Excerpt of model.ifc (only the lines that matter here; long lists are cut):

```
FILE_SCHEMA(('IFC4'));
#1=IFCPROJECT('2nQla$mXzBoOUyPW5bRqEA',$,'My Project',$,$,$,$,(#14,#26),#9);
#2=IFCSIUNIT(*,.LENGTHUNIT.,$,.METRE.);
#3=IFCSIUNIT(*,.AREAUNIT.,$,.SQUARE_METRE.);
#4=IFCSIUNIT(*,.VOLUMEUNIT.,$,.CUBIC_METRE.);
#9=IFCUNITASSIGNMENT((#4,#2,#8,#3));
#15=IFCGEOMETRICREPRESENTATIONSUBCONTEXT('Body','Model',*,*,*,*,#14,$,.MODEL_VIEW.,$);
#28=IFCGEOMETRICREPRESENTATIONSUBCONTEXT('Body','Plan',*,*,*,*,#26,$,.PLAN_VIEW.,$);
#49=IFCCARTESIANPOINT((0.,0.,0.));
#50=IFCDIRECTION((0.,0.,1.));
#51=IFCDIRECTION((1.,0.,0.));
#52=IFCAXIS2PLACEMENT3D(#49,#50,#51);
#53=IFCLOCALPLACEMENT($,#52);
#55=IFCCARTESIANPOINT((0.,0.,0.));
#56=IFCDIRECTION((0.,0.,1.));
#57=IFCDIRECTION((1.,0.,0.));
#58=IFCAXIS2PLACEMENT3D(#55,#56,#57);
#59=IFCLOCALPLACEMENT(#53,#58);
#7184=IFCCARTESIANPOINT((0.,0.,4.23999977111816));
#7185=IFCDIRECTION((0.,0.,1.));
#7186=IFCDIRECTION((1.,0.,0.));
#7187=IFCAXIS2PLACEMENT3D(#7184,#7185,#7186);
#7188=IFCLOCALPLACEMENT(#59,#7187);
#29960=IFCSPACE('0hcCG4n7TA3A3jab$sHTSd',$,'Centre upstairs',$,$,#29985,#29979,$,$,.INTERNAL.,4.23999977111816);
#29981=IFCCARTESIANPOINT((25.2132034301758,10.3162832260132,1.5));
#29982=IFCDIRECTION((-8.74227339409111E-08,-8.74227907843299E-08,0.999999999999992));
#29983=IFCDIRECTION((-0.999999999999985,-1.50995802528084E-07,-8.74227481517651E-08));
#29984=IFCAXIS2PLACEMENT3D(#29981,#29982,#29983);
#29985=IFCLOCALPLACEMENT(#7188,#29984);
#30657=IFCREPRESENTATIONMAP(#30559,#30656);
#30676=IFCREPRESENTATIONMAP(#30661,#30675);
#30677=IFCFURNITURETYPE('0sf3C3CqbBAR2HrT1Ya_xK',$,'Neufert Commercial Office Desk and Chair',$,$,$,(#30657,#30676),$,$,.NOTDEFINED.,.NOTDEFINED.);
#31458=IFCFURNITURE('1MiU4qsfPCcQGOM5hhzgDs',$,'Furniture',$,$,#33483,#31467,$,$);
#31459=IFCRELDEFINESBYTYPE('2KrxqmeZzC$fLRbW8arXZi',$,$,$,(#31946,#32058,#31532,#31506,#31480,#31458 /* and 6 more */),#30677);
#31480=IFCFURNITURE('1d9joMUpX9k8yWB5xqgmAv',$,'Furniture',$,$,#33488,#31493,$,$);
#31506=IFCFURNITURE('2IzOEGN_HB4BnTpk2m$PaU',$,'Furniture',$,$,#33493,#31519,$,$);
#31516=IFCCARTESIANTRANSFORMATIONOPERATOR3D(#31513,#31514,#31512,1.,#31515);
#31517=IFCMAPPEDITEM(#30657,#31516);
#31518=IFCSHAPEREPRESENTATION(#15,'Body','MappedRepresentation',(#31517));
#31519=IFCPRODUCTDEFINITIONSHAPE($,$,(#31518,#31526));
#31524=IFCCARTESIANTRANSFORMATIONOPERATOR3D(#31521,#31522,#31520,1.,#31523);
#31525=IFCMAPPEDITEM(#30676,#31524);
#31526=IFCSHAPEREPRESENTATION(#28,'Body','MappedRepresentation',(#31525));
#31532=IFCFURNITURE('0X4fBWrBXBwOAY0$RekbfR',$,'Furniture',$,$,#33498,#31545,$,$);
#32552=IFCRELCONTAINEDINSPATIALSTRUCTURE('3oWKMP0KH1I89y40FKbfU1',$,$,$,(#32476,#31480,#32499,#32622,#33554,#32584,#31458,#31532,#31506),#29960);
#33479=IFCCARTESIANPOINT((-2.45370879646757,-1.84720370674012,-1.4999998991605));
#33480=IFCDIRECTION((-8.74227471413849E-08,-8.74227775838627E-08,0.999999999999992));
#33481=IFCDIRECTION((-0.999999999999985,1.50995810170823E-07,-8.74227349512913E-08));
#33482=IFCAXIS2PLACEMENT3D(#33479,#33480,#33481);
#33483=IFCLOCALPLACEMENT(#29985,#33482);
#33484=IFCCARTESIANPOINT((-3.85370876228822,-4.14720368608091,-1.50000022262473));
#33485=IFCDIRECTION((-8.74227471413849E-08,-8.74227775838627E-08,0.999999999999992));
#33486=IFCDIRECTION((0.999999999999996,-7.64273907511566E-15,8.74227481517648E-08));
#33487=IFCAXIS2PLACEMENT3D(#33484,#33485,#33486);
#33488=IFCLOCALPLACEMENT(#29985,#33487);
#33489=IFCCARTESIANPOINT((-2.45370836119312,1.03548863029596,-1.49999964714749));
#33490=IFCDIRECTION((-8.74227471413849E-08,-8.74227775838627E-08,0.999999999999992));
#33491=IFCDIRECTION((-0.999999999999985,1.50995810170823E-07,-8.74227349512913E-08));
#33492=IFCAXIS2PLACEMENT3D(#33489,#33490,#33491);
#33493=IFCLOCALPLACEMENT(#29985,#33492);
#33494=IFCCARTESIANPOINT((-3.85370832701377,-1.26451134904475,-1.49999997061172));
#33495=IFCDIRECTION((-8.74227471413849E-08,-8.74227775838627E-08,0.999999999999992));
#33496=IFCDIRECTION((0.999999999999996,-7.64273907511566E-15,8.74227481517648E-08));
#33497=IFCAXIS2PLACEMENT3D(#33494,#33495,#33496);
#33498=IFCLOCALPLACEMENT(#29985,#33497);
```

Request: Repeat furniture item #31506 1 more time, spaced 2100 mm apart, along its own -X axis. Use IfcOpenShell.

```python
import ifcopenshell
import ifcopenshell.api.geometry
import ifcopenshell.api.root
import ifcopenshell.util.element
import ifcopenshell.util.placement

model = ifcopenshell.open("model.ifc")

source = model.by_guid("2IzOEGN_HB4BnTpk2m$PaU")
base = ifcopenshell.util.placement.get_local_placement(source.ObjectPlacement)
step = -base[:3, 0] * 2.1

for i in range(1, 2):
    copy = ifcopenshell.api.root.copy_class(model, product=source)
    copy.Representation = ifcopenshell.util.element.copy_deep(
        model, source.Representation, exclude=["IfcGeometricRepresentationContext", "IfcRepresentationMap"]
    )
    matrix = base.copy()
    matrix[:3, 3] += i * step
    print("added at", matrix[:3, 3].round(3) + 0.0)
    ifcopenshell.api.geometry.edit_object_placement(model, product=copy, matrix=matrix, is_si=False)

model.write("model_rev.ifc")
```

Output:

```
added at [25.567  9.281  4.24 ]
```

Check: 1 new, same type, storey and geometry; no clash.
